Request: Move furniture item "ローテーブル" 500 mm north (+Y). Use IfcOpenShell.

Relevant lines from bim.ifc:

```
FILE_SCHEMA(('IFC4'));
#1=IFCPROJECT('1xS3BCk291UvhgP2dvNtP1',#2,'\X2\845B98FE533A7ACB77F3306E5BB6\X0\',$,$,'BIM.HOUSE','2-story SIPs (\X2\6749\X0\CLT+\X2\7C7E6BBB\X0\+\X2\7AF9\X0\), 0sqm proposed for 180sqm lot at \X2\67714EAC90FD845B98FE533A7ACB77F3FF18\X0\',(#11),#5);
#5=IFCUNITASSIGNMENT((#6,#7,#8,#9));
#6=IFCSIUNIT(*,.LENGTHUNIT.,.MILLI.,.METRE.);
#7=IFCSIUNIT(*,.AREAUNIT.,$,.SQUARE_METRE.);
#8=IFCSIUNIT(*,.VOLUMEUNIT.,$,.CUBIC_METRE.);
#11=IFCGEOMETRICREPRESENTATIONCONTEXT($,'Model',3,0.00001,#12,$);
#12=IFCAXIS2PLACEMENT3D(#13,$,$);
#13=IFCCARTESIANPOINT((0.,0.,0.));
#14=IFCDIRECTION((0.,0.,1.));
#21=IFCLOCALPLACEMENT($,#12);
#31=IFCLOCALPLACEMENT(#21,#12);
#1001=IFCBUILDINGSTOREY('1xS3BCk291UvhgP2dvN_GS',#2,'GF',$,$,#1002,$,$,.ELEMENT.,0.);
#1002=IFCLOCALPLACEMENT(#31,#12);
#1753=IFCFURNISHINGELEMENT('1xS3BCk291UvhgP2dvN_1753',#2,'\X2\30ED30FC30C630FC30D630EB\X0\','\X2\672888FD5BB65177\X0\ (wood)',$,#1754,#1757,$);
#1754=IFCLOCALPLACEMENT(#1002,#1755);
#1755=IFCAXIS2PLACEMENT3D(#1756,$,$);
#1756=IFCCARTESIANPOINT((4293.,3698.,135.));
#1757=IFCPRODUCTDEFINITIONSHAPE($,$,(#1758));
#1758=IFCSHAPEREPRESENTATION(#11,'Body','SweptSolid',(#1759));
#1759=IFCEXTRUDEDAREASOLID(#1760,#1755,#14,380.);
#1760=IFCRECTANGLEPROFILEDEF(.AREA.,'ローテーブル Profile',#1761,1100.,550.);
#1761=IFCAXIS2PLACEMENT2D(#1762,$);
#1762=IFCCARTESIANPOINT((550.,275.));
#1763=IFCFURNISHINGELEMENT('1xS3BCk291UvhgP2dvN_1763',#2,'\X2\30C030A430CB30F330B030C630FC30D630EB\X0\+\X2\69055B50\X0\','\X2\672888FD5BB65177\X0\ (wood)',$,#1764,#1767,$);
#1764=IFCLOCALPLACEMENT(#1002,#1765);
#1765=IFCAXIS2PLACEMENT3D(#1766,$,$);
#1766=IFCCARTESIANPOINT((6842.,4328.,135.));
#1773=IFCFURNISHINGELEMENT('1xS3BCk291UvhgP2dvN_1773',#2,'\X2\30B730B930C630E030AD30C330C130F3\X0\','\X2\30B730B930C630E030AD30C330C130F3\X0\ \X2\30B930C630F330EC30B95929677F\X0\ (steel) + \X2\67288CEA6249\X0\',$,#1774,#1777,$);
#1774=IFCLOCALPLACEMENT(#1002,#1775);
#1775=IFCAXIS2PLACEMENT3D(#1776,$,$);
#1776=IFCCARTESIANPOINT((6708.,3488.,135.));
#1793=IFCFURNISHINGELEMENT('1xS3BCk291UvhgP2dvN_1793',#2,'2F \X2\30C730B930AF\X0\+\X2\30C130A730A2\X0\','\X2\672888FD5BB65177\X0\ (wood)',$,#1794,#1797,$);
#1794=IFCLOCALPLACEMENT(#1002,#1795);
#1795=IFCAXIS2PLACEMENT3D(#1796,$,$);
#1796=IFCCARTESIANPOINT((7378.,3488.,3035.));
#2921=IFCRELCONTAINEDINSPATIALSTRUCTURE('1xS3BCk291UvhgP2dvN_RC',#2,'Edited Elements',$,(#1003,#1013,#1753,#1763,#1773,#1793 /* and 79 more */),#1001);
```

```python
import ifcopenshell
import ifcopenshell.api.geometry
import ifcopenshell.util.placement
import ifcopenshell.util.unit

model = ifcopenshell.open("bim.ifc")
unit_scale = ifcopenshell.util.unit.calculate_unit_scale(model)

item = model.by_guid("1xS3BCk291UvhgP2dvN_1753")
matrix = ifcopenshell.util.placement.get_local_placement(item.ObjectPlacement)
matrix[1, 3] += 0.5 / unit_scale
ifcopenshell.api.geometry.edit_object_placement(model, product=item, matrix=matrix, is_si=False)

print(ifcopenshell.util.placement.get_local_placement(item.ObjectPlacement).round(3) + 0.0)

model.write("bim-out.ifc")
```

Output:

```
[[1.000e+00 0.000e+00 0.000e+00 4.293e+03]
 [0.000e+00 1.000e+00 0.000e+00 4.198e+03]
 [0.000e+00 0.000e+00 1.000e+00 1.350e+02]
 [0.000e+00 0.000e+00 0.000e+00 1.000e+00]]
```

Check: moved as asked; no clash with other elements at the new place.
